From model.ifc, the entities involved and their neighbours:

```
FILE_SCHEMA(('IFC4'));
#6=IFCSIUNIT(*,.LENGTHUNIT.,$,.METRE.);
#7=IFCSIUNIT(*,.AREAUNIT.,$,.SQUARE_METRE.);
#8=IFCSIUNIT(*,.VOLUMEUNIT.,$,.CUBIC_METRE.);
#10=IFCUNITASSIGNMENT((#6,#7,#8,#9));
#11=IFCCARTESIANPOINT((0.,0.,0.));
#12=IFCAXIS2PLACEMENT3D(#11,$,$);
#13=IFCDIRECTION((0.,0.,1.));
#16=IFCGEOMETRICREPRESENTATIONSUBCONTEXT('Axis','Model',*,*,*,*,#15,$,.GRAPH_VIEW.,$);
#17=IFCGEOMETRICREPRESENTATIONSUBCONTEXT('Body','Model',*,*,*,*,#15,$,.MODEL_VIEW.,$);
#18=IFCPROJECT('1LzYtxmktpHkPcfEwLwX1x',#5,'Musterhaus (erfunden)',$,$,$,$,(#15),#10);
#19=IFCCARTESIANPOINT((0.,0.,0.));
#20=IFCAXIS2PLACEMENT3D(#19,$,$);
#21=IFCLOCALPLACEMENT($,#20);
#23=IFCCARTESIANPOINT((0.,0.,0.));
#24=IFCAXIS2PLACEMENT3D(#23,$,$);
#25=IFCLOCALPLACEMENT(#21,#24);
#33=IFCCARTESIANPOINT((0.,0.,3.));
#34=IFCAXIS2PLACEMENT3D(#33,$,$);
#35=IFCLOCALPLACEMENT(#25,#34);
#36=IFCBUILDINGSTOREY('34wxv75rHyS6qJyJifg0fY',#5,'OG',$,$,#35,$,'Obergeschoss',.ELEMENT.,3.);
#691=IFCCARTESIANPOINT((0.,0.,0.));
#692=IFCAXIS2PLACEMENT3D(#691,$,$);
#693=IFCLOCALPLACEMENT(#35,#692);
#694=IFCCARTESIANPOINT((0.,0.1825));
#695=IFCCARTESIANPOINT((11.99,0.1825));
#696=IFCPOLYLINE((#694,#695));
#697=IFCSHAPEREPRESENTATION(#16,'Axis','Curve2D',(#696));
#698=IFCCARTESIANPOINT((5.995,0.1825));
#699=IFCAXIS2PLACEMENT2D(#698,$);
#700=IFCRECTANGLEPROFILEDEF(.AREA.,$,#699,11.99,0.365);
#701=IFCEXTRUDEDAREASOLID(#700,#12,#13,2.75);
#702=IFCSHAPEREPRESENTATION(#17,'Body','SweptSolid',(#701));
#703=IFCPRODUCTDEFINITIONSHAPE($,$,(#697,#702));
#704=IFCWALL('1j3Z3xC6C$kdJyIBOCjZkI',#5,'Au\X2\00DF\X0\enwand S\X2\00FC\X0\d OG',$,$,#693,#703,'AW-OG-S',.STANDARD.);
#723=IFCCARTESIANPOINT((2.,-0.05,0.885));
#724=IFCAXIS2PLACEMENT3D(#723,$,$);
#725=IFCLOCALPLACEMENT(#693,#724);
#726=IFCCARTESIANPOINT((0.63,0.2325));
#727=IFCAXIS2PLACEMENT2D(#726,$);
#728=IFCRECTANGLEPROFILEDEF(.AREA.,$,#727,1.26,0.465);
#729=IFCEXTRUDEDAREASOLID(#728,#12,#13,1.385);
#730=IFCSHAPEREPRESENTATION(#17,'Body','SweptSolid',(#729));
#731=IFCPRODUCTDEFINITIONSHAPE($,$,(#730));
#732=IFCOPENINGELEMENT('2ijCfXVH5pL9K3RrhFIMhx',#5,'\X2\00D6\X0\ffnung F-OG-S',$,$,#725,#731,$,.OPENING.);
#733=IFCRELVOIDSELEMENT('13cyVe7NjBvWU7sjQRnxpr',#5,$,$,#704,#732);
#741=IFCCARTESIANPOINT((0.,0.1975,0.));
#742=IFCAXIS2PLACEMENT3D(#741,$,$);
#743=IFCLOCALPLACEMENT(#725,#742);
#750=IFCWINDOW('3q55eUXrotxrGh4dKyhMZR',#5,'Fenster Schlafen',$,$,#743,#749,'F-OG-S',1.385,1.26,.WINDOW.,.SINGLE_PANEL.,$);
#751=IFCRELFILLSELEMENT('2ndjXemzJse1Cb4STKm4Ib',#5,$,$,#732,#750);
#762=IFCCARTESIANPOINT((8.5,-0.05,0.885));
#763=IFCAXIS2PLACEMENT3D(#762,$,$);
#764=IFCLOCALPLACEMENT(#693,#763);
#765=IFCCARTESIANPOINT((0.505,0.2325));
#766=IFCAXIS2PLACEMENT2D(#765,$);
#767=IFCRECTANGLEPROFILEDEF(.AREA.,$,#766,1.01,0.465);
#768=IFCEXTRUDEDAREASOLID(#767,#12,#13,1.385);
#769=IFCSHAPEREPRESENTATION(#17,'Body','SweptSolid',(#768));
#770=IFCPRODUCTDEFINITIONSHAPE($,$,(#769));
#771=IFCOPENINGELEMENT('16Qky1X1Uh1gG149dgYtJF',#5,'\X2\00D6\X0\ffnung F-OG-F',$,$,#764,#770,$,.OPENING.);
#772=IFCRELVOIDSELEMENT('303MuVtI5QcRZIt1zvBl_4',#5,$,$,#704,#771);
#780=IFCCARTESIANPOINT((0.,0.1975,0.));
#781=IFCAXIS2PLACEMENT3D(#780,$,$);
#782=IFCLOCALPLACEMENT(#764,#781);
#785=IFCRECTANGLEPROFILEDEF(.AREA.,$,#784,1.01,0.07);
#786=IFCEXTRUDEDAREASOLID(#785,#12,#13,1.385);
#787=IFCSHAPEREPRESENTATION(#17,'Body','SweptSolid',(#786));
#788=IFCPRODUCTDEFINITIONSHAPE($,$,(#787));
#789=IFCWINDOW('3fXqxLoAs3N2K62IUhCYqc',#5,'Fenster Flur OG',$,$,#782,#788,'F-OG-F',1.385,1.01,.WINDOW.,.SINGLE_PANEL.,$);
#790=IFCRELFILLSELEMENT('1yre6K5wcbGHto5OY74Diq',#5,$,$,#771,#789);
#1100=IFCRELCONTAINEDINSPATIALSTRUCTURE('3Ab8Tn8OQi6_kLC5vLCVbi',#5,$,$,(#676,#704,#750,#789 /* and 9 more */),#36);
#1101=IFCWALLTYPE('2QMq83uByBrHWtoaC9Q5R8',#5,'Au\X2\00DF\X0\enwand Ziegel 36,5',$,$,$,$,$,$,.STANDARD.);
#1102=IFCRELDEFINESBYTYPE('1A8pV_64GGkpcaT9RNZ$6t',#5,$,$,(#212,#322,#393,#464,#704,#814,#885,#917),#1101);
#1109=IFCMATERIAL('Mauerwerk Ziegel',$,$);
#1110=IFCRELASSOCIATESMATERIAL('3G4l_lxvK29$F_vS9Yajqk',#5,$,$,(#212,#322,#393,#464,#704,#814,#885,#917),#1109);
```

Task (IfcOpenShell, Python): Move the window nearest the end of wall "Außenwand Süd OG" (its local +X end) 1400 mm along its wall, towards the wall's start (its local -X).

```python
import ifcopenshell
import ifcopenshell.api.geometry
import ifcopenshell.util.placement
import ifcopenshell.util.unit

model = ifcopenshell.open("model.ifc")
unit_scale = ifcopenshell.util.unit.calculate_unit_scale(model)

window = model.by_guid("3fXqxLoAs3N2K62IUhCYqc")
opening = window.FillsVoids[0].RelatingOpeningElement
wall = opening.VoidsElements[0].RelatingBuildingElement

wall_matrix = ifcopenshell.util.placement.get_local_placement(wall.ObjectPlacement)
shift = wall_matrix[:3, 0] * -1.4 / unit_scale
before = ifcopenshell.util.placement.get_local_placement(window.ObjectPlacement)[:3, 3].copy()

# The window is placed relative to its opening, so it follows when the opening moves.
matrix = ifcopenshell.util.placement.get_local_placement(opening.ObjectPlacement)
matrix[:3, 3] += shift
ifcopenshell.api.geometry.edit_object_placement(
    model, product=opening, matrix=matrix, is_si=False, should_transform_children=True
)

after = ifcopenshell.util.placement.get_local_placement(window.ObjectPlacement)[:3, 3]
print("window moved by", (after - before).round(3) + 0.0)

model.write("model_edited.ifc")
```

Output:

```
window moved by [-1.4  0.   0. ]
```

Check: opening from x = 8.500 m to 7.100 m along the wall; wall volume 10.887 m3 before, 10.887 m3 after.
